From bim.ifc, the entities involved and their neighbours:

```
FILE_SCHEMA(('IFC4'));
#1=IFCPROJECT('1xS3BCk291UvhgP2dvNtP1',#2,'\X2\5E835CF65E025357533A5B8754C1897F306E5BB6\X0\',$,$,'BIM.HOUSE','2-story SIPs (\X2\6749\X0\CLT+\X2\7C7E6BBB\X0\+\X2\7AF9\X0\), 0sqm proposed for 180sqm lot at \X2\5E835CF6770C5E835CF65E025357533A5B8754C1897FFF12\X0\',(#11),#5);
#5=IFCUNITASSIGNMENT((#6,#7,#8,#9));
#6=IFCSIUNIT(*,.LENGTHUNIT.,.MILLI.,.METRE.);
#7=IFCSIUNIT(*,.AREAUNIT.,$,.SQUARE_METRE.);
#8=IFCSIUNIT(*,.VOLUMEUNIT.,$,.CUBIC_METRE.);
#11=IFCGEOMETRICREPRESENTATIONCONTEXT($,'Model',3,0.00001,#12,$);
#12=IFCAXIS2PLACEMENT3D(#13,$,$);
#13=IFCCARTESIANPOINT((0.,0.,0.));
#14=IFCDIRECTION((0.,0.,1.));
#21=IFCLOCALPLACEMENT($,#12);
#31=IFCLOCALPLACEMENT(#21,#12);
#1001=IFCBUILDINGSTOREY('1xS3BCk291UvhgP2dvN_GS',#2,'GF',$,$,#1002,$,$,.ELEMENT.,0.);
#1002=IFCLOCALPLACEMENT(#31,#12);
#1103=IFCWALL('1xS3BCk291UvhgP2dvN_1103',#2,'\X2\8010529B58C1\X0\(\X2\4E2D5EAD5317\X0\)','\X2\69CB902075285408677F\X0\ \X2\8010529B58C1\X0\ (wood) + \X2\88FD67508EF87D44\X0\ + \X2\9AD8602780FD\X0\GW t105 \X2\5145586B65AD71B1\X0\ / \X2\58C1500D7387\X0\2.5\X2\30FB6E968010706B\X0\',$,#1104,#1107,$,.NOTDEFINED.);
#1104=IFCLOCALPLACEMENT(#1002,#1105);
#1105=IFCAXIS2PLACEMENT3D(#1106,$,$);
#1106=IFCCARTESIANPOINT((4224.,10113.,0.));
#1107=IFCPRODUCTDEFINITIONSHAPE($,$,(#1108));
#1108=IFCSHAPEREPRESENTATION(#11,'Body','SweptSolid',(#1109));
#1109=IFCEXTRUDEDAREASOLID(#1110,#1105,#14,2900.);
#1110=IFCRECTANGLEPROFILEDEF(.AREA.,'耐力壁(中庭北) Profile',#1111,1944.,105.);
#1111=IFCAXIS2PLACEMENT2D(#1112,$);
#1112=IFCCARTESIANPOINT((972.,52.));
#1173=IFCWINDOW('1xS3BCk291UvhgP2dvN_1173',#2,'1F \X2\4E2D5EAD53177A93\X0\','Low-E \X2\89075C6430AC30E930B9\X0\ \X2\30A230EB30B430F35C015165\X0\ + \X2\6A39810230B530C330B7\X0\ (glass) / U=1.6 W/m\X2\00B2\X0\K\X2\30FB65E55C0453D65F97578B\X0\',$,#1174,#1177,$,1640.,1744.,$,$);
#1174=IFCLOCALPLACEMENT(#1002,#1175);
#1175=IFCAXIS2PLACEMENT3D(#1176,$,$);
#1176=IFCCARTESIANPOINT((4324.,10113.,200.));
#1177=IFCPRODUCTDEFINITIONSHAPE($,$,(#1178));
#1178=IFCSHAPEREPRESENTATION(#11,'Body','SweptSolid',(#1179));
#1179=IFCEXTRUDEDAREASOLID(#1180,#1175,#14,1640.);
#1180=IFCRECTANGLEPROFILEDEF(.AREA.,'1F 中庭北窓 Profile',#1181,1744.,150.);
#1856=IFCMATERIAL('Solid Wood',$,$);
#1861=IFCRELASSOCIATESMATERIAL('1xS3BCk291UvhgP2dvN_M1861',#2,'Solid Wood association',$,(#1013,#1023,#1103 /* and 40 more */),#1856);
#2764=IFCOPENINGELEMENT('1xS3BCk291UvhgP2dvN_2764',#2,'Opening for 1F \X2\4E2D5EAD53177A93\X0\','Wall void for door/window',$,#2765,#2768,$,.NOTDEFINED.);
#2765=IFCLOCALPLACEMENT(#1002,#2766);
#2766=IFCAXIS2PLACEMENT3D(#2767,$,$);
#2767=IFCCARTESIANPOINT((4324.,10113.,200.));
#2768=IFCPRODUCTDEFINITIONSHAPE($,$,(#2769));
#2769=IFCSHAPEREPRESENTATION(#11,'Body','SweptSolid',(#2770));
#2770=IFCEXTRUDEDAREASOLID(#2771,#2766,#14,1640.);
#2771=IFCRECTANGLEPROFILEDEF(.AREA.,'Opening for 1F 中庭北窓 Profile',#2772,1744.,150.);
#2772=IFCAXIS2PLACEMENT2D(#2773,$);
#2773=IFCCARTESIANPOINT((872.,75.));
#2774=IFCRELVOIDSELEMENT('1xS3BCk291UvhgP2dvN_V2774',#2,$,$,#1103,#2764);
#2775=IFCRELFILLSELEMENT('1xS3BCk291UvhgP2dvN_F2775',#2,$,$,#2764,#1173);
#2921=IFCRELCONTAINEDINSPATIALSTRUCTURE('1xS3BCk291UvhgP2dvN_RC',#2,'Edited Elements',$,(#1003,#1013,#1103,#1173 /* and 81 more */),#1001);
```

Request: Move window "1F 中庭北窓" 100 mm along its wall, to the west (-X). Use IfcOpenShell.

```python
import ifcopenshell
import ifcopenshell.api.geometry
import ifcopenshell.util.placement
import ifcopenshell.util.unit

model = ifcopenshell.open("bim.ifc")
unit_scale = ifcopenshell.util.unit.calculate_unit_scale(model)

window = model.by_guid("1xS3BCk291UvhgP2dvN_1173")
opening = window.FillsVoids[0].RelatingOpeningElement
wall = opening.VoidsElements[0].RelatingBuildingElement

wall_matrix = ifcopenshell.util.placement.get_local_placement(wall.ObjectPlacement)
shift = wall_matrix[:3, 0] * -0.1 / unit_scale
before = ifcopenshell.util.placement.get_local_placement(window.ObjectPlacement)[:3, 3].copy()

# The window is not placed relative to its opening, so move both.
for product in (opening, window):
    matrix = ifcopenshell.util.placement.get_local_placement(product.ObjectPlacement)
    matrix[:3, 3] += shift
    ifcopenshell.api.geometry.edit_object_placement(model, product=product, matrix=matrix, is_si=False)

after = ifcopenshell.util.placement.get_local_placement(window.ObjectPlacement)[:3, 3]
print("window moved by", (after - before).round(3) + 0.0)

model.write("bim_updated.ifc")
```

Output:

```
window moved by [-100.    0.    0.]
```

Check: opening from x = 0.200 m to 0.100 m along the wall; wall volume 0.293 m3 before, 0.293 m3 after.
